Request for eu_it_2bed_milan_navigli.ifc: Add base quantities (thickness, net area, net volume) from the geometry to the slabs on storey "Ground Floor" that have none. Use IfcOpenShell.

First a look at what the model holds.

```python
import ifcopenshell
import ifcopenshell.util.element
import ifcopenshell.util.unit

model = ifcopenshell.open("eu_it_2bed_milan_navigli.ifc")
print(model.schema)
for unit_type in ("LENGTHUNIT", "AREAUNIT", "VOLUMEUNIT"):
    print(unit_type, ifcopenshell.util.unit.calculate_unit_scale(model, unit_type))
storey = next(s for s in model.by_type("IfcBuildingStorey") if s.Name == "Ground Floor")
slabs = [e for e in ifcopenshell.util.element.get_decomposition(storey) if e.is_a("IfcSlab")]
for e in sorted(slabs, key=lambda e: e.id()):
    print(e.id(), e.is_a(), e.Name, list(ifcopenshell.util.element.get_psets(e, qtos_only=True)), sep=" | ")
```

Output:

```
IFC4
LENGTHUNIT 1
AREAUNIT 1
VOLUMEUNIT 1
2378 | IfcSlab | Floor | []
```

```python
import ifcopenshell
import ifcopenshell.api.pset
import ifcopenshell.geom
import ifcopenshell.util.element
import ifcopenshell.util.shape
import ifcopenshell.util.unit

model = ifcopenshell.open("eu_it_2bed_milan_navigli.ifc")
unit_scale = ifcopenshell.util.unit.calculate_unit_scale(model)
area_scale = ifcopenshell.util.unit.calculate_unit_scale(model, "AREAUNIT")
volume_scale = ifcopenshell.util.unit.calculate_unit_scale(model, "VOLUMEUNIT")
settings = ifcopenshell.geom.settings()

storey = next(s for s in model.by_type("IfcBuildingStorey") if s.Name == "Ground Floor")
slabs = [e for e in ifcopenshell.util.element.get_decomposition(storey) if e.is_a("IfcSlab")]

for e in sorted(slabs, key=lambda e: e.id()):
    if ifcopenshell.util.element.get_psets(e, qtos_only=True, should_inherit=False):
        continue
    # Geometry comes back in metres, in the element's own axes.
    shape = ifcopenshell.geom.create_shape(settings, e)
    values = {
        "Width": ifcopenshell.util.shape.get_z(shape.geometry) / unit_scale,
        "NetArea": ifcopenshell.util.shape.get_footprint_area(shape.geometry) / area_scale,
        "NetVolume": ifcopenshell.util.shape.get_volume(shape.geometry) / volume_scale,
    }
    qto = ifcopenshell.api.pset.add_qto(model, product=e, name="Qto_SlabBaseQuantities")
    ifcopenshell.api.pset.edit_qto(model, qto=qto, properties=values)
    print(e.id(), {k: round(v, 3) for k, v in values.items()})

model.write("eu_it_2bed_milan_navigli_edited.ifc")
```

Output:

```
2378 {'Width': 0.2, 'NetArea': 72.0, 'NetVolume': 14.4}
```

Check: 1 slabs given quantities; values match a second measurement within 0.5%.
